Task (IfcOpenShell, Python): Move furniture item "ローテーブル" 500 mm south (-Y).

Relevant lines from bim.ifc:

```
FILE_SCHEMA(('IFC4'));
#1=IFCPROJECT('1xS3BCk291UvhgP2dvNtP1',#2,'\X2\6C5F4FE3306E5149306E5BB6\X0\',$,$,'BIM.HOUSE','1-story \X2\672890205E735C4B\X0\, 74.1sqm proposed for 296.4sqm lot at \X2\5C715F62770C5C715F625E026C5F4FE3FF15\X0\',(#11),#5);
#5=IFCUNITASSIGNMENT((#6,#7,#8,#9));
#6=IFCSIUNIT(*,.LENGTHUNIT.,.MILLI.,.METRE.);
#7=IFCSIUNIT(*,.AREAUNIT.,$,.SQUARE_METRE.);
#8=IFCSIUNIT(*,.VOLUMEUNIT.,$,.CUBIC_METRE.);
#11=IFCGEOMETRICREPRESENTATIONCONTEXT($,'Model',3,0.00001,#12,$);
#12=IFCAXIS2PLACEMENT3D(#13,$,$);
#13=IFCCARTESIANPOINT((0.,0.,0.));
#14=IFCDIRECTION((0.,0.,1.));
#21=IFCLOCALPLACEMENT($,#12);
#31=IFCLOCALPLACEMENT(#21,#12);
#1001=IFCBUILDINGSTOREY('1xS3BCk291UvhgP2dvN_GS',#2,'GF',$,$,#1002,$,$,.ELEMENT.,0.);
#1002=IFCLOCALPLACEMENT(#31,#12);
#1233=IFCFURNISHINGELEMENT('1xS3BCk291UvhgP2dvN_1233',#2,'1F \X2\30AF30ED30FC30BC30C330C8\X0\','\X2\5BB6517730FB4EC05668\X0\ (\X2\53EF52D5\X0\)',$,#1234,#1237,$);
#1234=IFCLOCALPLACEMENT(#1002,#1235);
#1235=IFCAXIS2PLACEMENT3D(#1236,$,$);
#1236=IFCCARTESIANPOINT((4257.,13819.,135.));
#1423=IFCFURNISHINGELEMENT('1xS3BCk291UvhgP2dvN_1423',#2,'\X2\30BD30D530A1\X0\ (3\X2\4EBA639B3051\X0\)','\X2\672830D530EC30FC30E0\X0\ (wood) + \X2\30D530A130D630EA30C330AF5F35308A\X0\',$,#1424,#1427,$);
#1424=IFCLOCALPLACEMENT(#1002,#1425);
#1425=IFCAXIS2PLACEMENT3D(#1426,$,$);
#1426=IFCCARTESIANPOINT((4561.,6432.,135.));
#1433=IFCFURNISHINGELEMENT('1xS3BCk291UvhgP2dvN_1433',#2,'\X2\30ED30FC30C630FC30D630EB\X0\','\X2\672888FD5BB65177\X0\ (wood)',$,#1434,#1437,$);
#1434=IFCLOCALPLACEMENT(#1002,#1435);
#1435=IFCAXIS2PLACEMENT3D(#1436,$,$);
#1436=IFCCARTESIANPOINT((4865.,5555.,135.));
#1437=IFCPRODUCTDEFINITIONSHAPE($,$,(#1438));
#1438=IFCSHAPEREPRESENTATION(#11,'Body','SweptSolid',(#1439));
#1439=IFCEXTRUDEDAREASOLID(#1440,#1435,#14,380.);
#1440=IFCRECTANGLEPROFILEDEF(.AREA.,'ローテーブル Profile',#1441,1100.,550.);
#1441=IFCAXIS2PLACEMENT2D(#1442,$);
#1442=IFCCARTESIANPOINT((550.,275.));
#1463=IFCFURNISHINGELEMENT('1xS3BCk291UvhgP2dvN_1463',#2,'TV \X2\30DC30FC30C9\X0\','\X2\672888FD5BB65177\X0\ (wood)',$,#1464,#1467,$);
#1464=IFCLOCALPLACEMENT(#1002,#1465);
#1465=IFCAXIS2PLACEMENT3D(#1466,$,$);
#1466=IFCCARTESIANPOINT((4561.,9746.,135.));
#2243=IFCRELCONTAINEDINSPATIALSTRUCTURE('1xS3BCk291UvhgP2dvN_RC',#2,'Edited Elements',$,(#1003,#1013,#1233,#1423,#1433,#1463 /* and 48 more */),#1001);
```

```python
import ifcopenshell
import ifcopenshell.api.geometry
import ifcopenshell.util.placement
import ifcopenshell.util.unit

model = ifcopenshell.open("bim.ifc")
unit_scale = ifcopenshell.util.unit.calculate_unit_scale(model)

item = model.by_guid("1xS3BCk291UvhgP2dvN_1433")
matrix = ifcopenshell.util.placement.get_local_placement(item.ObjectPlacement)
matrix[1, 3] -= 0.5 / unit_scale
ifcopenshell.api.geometry.edit_object_placement(model, product=item, matrix=matrix, is_si=False)

print(ifcopenshell.util.placement.get_local_placement(item.ObjectPlacement).round(3) + 0.0)

model.write("bim_rev.ifc")
```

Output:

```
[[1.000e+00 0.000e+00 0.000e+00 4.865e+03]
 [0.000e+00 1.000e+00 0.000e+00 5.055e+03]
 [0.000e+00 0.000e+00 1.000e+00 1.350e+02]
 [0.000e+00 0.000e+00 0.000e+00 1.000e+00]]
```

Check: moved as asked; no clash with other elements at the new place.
